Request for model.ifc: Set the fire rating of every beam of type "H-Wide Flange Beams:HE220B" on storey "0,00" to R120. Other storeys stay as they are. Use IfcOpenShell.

First a look at what the model holds.

```python
import ifcopenshell
import ifcopenshell.util.element

model = ifcopenshell.open("model.ifc")
print(model.schema)
storey = next(s for s in model.by_type("IfcBuildingStorey") if s.Name == "0,00")
beams = [e for e in ifcopenshell.util.element.get_decomposition(storey) if e.is_a("IfcBeam")]
seen = {}
for e in beams:
    element_type = ifcopenshell.util.element.get_type(e)
    key = (element_type.Name if element_type != e and element_type else None, ifcopenshell.util.element.get_pset(e, "Pset_BeamCommon", "FireRating"))
    seen[key] = seen.get(key, 0) + 1
for (name, value), count in sorted(seen.items(), key=str):
    print(count, "x", name, "|", value)
```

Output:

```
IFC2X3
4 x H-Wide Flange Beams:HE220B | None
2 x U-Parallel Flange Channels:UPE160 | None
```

```python
import ifcopenshell
import ifcopenshell.api.pset
import ifcopenshell.util.element

model = ifcopenshell.open("model.ifc")

storey = next(s for s in model.by_type("IfcBuildingStorey") if s.Name == "0,00")
beams = [e for e in ifcopenshell.util.element.get_decomposition(storey) if e.is_a("IfcBeam")]

count = 0
for e in beams:
    element_type = ifcopenshell.util.element.get_type(e)
    if element_type in (None, e) or element_type.Name != "H-Wide Flange Beams:HE220B":
        continue
    # add_pset returns the element's existing set when there is one.
    pset = ifcopenshell.api.pset.add_pset(model, product=e, name="Pset_BeamCommon")
    ifcopenshell.api.pset.edit_pset(model, pset=pset, properties={"FireRating": "R120"})
    count += 1

print(count, "beams updated")

model.write("model-out.ifc")
```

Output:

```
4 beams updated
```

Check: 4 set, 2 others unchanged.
